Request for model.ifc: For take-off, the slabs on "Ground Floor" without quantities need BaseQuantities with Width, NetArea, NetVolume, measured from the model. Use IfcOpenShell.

First a look at what the model holds.

```python
import ifcopenshell
import ifcopenshell.util.element
import ifcopenshell.util.unit

model = ifcopenshell.open("model.ifc")
print(model.schema)
for unit_type in ("LENGTHUNIT", "AREAUNIT", "VOLUMEUNIT"):
    print(unit_type, ifcopenshell.util.unit.calculate_unit_scale(model, unit_type))
storey = next(s for s in model.by_type("IfcBuildingStorey") if s.Name == "Ground Floor")
slabs = [e for e in ifcopenshell.util.element.get_decomposition(storey) if e.is_a("IfcSlab")]
for e in sorted(slabs, key=lambda e: e.id()):
    print(e.id(), e.is_a(), e.Name, list(ifcopenshell.util.element.get_psets(e, qtos_only=True)), sep=" | ")
```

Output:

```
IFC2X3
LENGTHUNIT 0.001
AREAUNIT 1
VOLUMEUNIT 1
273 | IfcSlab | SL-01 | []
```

```python
import ifcopenshell
import ifcopenshell.api.pset
import ifcopenshell.geom
import ifcopenshell.util.element
import ifcopenshell.util.shape
import ifcopenshell.util.unit

model = ifcopenshell.open("model.ifc")
unit_scale = ifcopenshell.util.unit.calculate_unit_scale(model)
area_scale = ifcopenshell.util.unit.calculate_unit_scale(model, "AREAUNIT")
volume_scale = ifcopenshell.util.unit.calculate_unit_scale(model, "VOLUMEUNIT")
settings = ifcopenshell.geom.settings()

storey = next(s for s in model.by_type("IfcBuildingStorey") if s.Name == "Ground Floor")
slabs = [e for e in ifcopenshell.util.element.get_decomposition(storey) if e.is_a("IfcSlab")]

for e in sorted(slabs, key=lambda e: e.id()):
    if ifcopenshell.util.element.get_psets(e, qtos_only=True, should_inherit=False):
        continue
    # Geometry comes back in metres, in the element's own axes.
    shape = ifcopenshell.geom.create_shape(settings, e)
    values = {
        "Width": ifcopenshell.util.shape.get_z(shape.geometry) / unit_scale,
        "NetArea": ifcopenshell.util.shape.get_footprint_area(shape.geometry) / area_scale,
        "NetVolume": ifcopenshell.util.shape.get_volume(shape.geometry) / volume_scale,
    }
    qto = ifcopenshell.api.pset.add_qto(model, product=e, name="BaseQuantities")
    ifcopenshell.api.pset.edit_qto(model, qto=qto, properties=values)
    print(e.id(), {k: round(v, 3) for k, v in values.items()})

model.write("model-out.ifc")
```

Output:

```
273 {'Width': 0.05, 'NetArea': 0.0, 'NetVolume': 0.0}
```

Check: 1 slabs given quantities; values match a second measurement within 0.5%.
